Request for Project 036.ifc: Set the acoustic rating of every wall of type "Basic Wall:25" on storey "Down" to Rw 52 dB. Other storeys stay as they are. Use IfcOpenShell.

First a look at what the model holds.

```python
import ifcopenshell
import ifcopenshell.util.element

model = ifcopenshell.open("Project 036.ifc")
print(model.schema)
storey = next(s for s in model.by_type("IfcBuildingStorey") if s.Name == "Down")
walls = [e for e in ifcopenshell.util.element.get_decomposition(storey) if e.is_a("IfcWall")]
seen = {}
for e in walls:
    element_type = ifcopenshell.util.element.get_type(e)
    key = (element_type.Name if element_type != e and element_type else None, ifcopenshell.util.element.get_pset(e, "Pset_WallCommon", "AcousticRating"))
    seen[key] = seen.get(key, 0) + 1
for (name, value), count in sorted(seen.items(), key=str):
    print(count, "x", name, "|", value)
```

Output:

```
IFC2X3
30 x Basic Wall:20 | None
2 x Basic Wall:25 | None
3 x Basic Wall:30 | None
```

```python
import ifcopenshell
import ifcopenshell.api.pset
import ifcopenshell.util.element

model = ifcopenshell.open("Project 036.ifc")

storey = next(s for s in model.by_type("IfcBuildingStorey") if s.Name == "Down")
walls = [e for e in ifcopenshell.util.element.get_decomposition(storey) if e.is_a("IfcWall")]

count = 0
for e in walls:
    element_type = ifcopenshell.util.element.get_type(e)
    if element_type in (None, e) or element_type.Name != "Basic Wall:25":
        continue
    # add_pset returns the element's existing set when there is one.
    pset = ifcopenshell.api.pset.add_pset(model, product=e, name="Pset_WallCommon")
    ifcopenshell.api.pset.edit_pset(model, pset=pset, properties={"AcousticRating": "Rw 52 dB"})
    count += 1

print(count, "walls updated")

model.write("Project 036_rev.ifc")
```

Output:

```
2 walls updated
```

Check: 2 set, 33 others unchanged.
